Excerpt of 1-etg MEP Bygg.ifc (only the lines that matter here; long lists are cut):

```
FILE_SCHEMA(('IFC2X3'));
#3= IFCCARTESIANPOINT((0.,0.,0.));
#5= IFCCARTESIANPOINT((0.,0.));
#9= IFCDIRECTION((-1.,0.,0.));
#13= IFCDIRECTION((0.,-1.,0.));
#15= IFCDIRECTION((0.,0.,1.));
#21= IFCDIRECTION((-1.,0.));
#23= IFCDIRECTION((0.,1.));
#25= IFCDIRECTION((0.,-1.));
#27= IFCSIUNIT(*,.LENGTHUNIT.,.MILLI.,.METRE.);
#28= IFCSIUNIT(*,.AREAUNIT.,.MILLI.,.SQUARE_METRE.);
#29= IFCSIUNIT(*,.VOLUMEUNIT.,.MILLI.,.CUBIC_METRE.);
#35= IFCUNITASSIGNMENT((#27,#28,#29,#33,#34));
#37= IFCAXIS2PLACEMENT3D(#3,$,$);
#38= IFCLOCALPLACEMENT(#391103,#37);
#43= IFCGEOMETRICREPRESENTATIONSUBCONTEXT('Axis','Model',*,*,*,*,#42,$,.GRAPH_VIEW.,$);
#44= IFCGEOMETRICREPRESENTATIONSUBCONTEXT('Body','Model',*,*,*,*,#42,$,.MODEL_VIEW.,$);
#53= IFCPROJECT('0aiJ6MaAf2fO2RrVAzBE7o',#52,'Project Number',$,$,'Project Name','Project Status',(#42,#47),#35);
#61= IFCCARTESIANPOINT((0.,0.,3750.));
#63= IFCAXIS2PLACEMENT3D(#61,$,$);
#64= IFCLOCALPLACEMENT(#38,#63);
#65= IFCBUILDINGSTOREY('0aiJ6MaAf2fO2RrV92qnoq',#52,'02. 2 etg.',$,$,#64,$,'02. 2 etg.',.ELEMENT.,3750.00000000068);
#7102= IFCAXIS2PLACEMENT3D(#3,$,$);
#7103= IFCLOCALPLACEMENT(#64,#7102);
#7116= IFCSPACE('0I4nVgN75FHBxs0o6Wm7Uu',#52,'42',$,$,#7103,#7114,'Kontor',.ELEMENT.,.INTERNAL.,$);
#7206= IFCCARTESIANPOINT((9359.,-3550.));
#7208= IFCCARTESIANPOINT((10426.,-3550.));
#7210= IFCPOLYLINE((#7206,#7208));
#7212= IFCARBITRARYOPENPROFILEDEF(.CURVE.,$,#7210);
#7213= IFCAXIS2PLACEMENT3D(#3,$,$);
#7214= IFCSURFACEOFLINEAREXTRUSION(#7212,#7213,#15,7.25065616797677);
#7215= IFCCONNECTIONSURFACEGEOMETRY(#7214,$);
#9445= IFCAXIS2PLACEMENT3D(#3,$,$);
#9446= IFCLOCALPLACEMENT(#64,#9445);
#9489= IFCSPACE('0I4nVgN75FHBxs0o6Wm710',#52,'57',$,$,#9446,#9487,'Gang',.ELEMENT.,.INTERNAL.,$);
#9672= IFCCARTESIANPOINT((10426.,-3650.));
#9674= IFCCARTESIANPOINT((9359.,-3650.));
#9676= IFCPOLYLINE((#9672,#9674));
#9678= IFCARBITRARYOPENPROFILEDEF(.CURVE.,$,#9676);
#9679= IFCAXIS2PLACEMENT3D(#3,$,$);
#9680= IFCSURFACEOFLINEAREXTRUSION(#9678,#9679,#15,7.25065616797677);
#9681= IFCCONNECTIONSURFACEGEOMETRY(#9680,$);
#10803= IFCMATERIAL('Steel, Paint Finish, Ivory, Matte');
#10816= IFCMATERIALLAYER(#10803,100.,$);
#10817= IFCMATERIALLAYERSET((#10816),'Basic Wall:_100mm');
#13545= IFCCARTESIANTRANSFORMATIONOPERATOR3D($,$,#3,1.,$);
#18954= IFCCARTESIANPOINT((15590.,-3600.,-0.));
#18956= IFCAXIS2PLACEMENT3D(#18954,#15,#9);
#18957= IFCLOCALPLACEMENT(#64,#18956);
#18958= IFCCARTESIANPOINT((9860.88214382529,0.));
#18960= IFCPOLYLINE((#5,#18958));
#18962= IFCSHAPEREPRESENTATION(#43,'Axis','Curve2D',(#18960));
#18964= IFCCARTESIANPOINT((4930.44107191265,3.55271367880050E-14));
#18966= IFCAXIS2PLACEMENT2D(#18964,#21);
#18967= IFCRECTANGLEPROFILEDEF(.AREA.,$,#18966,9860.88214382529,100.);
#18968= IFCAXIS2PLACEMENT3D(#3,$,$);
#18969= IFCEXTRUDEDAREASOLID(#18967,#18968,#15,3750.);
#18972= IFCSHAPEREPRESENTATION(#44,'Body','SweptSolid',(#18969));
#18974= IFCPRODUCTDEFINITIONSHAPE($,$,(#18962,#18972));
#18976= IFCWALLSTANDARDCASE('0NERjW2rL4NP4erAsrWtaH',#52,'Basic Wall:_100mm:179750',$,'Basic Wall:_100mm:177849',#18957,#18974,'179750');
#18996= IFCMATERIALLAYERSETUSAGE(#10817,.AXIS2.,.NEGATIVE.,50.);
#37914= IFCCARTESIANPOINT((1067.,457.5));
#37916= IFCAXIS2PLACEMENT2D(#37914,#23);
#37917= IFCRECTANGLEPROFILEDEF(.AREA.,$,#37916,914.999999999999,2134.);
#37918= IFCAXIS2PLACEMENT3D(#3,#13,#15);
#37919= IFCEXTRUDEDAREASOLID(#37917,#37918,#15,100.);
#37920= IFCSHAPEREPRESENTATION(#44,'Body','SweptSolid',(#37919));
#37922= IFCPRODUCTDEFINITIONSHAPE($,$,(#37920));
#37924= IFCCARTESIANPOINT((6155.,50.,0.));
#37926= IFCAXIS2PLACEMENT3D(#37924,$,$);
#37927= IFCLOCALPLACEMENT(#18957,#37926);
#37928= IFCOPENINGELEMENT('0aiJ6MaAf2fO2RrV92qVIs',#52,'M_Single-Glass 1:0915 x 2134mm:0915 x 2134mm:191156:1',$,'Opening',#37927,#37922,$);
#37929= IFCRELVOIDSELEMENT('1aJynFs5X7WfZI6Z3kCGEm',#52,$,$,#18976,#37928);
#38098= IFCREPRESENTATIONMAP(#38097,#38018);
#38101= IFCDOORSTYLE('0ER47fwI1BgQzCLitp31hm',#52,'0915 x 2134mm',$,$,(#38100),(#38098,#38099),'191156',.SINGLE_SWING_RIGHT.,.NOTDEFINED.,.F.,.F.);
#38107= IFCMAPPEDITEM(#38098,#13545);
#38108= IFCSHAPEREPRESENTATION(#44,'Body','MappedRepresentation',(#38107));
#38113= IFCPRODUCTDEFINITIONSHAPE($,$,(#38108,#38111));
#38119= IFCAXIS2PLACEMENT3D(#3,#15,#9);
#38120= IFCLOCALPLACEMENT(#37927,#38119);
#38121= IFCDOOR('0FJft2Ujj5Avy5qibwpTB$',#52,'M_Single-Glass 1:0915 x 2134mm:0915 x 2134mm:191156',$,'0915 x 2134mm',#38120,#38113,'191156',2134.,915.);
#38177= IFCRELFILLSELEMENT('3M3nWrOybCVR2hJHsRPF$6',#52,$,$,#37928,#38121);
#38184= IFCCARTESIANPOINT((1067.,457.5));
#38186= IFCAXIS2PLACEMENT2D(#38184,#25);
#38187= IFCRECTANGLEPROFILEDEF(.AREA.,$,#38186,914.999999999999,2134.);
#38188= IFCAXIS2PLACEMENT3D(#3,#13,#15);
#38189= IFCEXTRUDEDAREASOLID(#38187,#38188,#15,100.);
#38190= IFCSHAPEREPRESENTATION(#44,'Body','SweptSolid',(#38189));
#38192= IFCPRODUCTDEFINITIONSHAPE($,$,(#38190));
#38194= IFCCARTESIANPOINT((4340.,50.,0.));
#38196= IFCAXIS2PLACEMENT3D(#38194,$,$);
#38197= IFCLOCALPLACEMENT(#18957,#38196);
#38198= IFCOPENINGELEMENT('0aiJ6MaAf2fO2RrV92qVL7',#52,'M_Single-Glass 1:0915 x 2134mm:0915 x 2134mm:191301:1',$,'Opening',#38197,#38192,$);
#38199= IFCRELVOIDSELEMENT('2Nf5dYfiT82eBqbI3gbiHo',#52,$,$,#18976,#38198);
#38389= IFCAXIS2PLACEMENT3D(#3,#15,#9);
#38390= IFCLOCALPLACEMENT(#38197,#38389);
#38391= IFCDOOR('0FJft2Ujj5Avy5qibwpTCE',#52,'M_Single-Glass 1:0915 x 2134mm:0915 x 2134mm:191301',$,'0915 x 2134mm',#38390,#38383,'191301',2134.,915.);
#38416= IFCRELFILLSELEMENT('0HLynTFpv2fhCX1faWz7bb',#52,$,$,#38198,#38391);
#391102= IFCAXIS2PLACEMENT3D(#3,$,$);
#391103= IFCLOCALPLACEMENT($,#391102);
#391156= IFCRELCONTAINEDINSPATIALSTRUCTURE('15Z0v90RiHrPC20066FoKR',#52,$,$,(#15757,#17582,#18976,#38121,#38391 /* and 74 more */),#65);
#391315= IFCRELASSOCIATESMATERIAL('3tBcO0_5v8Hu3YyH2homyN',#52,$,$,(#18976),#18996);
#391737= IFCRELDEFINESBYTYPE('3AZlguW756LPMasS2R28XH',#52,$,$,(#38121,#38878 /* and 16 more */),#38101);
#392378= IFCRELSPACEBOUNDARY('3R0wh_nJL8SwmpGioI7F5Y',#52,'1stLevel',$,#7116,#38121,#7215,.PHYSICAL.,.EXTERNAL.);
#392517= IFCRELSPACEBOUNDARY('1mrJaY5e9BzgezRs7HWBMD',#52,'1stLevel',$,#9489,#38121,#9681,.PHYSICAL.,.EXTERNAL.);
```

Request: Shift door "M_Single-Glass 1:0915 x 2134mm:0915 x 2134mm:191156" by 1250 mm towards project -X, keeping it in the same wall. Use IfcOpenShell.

```python
import numpy as np
import ifcopenshell
import ifcopenshell.api.geometry
import ifcopenshell.util.placement

model = ifcopenshell.open("1-etg MEP Bygg.ifc")

door = model.by_guid("0FJft2Ujj5Avy5qibwpTB$")
opening = door.FillsVoids[0].RelatingOpeningElement
wall = opening.VoidsElements[0].RelatingBuildingElement

wall_matrix = ifcopenshell.util.placement.get_local_placement(wall.ObjectPlacement)
shift = wall_matrix[:3, 0] * 1250.0
before = ifcopenshell.util.placement.get_local_placement(door.ObjectPlacement)[:3, 3].copy()

# The door is placed relative to its opening, so it follows when the opening moves.
matrix = ifcopenshell.util.placement.get_local_placement(opening.ObjectPlacement)
matrix[:3, 3] += shift
ifcopenshell.api.geometry.edit_object_placement(
    model, product=opening, matrix=matrix, is_si=False, should_transform_children=True
)

# Space boundary surfaces are stored in each space's coordinates; move them too.
for rel in door.ProvidesBoundaries:
    if not rel.ConnectionGeometry:
        continue
    surface = rel.ConnectionGeometry.SurfaceOnRelatingElement
    space_matrix = ifcopenshell.util.placement.get_local_placement(rel.RelatingSpace.ObjectPlacement)
    point = np.array(surface.Position.Location.Coordinates) + space_matrix[:3, :3].T @ shift
    surface.Position = model.createIfcAxis2Placement3D(
        model.createIfcCartesianPoint(point.tolist()), surface.Position.Axis, surface.Position.RefDirection
    )

after = ifcopenshell.util.placement.get_local_placement(door.ObjectPlacement)[:3, 3]
print("door moved by", (after - before).round(3) + 0.0)

model.write("1-etg MEP Bygg-out.ifc")
```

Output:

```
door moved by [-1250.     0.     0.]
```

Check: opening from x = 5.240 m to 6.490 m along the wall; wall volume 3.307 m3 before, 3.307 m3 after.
